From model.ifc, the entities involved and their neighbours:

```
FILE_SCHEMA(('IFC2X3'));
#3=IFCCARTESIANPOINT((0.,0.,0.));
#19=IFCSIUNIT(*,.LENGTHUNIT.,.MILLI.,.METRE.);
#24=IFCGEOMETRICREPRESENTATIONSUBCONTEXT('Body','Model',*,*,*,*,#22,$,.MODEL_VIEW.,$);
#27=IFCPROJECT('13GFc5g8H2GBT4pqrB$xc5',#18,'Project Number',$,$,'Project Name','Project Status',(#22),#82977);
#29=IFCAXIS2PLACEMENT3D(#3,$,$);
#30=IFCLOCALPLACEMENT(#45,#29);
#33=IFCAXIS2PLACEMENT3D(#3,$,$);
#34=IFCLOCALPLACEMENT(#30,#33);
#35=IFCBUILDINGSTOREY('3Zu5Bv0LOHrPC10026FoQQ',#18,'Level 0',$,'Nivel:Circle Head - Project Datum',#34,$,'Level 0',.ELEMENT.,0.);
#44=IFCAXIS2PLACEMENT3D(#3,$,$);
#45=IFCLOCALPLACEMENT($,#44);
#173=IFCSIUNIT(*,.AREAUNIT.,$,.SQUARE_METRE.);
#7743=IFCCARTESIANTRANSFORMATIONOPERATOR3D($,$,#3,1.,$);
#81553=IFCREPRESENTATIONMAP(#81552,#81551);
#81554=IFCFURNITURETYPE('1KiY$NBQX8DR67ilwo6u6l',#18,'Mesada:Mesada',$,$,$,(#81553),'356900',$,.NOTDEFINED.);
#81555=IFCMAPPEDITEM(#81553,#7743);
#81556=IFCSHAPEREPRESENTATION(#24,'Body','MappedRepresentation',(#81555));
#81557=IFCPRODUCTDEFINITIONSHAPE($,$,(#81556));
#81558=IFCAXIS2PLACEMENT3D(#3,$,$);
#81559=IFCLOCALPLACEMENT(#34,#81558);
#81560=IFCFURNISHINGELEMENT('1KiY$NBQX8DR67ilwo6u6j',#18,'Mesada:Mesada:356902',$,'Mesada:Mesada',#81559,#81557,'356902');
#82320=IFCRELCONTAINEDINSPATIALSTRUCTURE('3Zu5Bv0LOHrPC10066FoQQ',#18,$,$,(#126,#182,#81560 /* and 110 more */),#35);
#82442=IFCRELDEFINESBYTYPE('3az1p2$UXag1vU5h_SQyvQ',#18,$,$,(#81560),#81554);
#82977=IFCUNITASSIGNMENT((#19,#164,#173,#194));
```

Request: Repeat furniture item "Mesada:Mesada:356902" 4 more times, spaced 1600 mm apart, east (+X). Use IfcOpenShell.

```python
import numpy as np
import ifcopenshell
import ifcopenshell.api.geometry
import ifcopenshell.api.root
import ifcopenshell.util.element
import ifcopenshell.util.placement
import ifcopenshell.util.unit

model = ifcopenshell.open("model.ifc")
unit_scale = ifcopenshell.util.unit.calculate_unit_scale(model)


def reuse_history(source, copy):
    """copy_class also copies each property set's owner history, people and application; keep the originals."""
    for rel in copy.IsDefinedBy:
        if rel.is_a("IfcRelDefinesByProperties") and (history := rel.RelatingPropertyDefinition.OwnerHistory):
            rel.RelatingPropertyDefinition.OwnerHistory = source.OwnerHistory
            ifcopenshell.util.element.remove_deep2(model, history)


source = model.by_guid("1KiY$NBQX8DR67ilwo6u6j")
base = ifcopenshell.util.placement.get_local_placement(source.ObjectPlacement)
step = np.array([1.0, 0.0, 0.0]) * 1.6 / unit_scale

for i in range(1, 5):
    copy = ifcopenshell.api.root.copy_class(model, product=source)
    copy.Representation = ifcopenshell.util.element.copy_deep(
        model, source.Representation, exclude=["IfcGeometricRepresentationContext", "IfcRepresentationMap"]
    )
    copy.Name = "Mesada:Mesada"
    copy.Tag = None
    reuse_history(source, copy)
    matrix = base.copy()
    matrix[:3, 3] += i * step
    print("added at", matrix[:3, 3].round(3) + 0.0)
    ifcopenshell.api.geometry.edit_object_placement(model, product=copy, matrix=matrix, is_si=False)

model.write("model_updated.ifc")
```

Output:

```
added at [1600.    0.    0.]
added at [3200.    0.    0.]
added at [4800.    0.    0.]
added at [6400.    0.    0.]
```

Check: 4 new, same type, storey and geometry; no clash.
